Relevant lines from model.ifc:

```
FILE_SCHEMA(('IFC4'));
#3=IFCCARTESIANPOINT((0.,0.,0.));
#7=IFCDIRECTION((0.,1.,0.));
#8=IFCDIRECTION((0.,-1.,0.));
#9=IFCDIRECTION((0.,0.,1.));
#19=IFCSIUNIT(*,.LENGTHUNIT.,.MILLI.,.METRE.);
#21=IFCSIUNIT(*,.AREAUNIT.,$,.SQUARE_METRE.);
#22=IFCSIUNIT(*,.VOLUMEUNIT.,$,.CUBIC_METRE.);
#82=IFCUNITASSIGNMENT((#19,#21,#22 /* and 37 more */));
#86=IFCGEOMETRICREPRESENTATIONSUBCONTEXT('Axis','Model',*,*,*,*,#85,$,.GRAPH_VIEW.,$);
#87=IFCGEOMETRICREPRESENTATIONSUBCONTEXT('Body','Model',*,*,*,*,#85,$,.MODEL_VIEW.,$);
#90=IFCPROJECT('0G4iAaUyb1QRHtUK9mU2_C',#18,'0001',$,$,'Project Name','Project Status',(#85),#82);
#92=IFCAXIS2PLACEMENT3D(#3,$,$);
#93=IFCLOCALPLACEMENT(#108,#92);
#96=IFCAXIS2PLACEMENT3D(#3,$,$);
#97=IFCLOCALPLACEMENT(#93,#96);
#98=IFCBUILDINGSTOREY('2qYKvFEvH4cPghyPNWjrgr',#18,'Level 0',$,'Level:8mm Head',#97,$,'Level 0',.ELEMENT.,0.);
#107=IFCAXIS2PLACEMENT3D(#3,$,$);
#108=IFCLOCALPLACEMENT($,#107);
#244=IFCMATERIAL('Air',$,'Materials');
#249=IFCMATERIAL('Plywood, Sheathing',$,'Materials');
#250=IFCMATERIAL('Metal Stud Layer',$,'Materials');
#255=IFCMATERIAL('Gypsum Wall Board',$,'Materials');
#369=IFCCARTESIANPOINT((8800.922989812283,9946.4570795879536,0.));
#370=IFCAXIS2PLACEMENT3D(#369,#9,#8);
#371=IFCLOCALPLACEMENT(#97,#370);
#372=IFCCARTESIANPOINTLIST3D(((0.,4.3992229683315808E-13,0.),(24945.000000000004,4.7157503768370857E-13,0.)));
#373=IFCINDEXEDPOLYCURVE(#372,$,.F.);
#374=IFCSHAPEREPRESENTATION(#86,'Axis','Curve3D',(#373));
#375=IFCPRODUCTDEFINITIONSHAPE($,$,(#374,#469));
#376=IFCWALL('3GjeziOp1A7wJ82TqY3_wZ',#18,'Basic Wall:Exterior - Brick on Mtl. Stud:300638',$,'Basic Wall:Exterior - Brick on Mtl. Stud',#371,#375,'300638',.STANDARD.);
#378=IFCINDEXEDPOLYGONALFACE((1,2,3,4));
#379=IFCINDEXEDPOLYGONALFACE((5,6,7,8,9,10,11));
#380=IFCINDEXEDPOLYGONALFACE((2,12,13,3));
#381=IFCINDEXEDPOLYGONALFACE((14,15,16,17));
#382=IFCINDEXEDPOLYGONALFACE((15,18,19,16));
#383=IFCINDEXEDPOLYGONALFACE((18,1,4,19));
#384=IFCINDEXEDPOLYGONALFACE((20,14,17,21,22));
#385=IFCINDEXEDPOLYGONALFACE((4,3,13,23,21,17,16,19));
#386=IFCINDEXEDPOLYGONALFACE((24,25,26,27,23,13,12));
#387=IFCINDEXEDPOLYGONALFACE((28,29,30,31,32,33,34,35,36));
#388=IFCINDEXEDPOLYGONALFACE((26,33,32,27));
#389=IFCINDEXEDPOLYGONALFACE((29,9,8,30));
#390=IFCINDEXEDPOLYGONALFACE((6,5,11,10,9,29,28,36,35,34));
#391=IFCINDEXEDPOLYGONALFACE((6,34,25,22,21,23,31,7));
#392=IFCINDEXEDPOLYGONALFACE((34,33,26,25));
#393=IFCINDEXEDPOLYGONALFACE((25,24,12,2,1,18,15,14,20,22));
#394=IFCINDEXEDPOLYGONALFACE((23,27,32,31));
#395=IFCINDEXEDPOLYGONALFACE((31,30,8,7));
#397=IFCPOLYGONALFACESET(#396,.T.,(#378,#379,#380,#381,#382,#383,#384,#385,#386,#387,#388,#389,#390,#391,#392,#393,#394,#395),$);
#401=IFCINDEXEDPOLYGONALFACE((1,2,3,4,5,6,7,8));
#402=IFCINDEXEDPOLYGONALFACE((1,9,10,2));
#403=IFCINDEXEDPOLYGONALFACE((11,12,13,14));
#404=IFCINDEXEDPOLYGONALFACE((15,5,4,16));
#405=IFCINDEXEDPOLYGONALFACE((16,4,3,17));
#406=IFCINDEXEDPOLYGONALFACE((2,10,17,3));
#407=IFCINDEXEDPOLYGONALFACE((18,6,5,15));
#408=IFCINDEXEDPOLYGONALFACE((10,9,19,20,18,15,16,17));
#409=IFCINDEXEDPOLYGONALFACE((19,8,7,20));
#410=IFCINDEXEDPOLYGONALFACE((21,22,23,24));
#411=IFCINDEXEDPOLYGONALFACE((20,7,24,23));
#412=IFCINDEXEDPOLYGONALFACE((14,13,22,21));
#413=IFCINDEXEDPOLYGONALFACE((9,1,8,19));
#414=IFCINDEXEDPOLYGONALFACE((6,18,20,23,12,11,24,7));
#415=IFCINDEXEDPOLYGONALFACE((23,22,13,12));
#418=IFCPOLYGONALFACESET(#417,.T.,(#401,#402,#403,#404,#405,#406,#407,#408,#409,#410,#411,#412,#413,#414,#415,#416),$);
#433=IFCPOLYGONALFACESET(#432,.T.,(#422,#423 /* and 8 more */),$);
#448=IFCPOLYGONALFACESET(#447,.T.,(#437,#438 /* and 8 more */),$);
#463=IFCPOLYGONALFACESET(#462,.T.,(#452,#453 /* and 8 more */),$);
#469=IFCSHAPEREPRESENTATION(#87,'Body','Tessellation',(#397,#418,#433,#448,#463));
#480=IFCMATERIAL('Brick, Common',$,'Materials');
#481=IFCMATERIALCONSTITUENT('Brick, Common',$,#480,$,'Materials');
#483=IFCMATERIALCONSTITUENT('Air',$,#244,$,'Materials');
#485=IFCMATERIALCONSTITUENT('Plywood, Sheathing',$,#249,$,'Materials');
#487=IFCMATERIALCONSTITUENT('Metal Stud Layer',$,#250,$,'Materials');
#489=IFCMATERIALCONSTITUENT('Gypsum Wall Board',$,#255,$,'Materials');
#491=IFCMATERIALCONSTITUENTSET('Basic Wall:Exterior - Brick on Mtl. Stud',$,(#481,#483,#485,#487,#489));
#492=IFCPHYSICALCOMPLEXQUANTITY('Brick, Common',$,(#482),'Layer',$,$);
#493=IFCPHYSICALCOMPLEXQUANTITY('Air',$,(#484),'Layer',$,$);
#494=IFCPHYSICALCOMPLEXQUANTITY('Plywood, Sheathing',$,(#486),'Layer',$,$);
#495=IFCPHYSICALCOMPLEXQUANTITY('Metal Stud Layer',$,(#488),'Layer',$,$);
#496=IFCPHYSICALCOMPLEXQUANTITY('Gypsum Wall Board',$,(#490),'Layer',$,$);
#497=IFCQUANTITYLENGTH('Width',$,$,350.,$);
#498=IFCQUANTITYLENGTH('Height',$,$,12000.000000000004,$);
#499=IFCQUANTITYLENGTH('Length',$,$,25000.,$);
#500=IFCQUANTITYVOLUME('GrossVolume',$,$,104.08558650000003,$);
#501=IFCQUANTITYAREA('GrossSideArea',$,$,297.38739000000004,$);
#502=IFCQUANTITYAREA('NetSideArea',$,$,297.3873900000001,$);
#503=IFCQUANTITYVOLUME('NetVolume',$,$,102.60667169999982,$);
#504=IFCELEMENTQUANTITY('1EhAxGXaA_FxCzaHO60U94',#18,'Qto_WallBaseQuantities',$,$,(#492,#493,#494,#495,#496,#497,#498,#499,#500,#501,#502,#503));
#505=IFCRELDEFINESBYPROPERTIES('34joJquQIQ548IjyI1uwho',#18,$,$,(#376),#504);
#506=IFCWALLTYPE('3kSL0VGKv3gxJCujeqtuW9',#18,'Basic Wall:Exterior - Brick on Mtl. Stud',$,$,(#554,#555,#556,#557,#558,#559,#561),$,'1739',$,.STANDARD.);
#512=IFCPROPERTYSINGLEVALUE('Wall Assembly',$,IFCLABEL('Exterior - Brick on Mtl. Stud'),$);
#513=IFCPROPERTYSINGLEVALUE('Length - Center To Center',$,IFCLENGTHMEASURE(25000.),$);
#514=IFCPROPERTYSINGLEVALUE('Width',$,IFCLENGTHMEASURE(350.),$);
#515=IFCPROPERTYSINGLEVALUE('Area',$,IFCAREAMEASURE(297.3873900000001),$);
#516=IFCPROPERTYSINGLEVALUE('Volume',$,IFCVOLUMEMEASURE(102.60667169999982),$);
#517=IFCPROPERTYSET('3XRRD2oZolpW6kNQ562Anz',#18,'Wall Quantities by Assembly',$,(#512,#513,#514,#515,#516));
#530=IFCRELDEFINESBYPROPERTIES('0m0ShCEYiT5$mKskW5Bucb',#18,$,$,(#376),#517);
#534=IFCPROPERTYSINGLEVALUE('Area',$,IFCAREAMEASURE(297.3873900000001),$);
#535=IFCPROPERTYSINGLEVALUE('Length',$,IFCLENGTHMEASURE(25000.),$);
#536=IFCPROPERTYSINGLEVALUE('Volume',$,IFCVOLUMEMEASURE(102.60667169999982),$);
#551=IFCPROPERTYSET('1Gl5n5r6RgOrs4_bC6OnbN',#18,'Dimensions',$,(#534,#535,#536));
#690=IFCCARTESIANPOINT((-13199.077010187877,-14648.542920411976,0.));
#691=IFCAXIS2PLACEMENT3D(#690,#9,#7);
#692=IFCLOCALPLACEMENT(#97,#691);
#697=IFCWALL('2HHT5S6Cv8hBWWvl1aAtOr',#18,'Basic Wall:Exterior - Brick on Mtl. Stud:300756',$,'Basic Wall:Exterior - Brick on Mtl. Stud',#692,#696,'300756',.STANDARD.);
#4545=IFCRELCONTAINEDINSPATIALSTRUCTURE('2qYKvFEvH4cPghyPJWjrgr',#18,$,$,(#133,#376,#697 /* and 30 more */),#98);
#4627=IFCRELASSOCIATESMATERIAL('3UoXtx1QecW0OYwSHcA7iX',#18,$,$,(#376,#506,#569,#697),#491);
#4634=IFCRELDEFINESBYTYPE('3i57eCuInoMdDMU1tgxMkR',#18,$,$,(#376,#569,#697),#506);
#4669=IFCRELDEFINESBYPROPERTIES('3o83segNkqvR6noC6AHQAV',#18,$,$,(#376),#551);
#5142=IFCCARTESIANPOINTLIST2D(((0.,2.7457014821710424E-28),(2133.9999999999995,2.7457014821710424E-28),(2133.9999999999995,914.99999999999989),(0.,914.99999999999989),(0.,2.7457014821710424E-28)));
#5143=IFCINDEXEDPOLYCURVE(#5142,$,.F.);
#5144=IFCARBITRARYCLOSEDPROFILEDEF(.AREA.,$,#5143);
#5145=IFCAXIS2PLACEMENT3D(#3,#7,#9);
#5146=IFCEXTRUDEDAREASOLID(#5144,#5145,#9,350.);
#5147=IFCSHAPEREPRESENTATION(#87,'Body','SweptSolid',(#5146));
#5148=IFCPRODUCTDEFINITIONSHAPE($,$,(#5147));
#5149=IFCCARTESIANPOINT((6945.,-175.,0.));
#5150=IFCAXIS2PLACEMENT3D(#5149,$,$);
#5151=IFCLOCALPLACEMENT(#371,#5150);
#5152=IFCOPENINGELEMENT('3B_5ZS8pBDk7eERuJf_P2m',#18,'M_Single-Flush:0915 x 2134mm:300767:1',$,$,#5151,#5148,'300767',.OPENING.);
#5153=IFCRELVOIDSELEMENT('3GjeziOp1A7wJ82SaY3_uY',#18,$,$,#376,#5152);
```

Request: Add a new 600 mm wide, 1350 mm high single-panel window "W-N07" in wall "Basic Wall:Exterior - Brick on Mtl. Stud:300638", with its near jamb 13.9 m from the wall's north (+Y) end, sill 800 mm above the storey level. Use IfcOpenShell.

```python
import numpy as np
import ifcopenshell
import ifcopenshell.api.feature
import ifcopenshell.api.geometry
import ifcopenshell.api.pset
import ifcopenshell.api.root
import ifcopenshell.api.spatial
import ifcopenshell.geom
import ifcopenshell.util.element
import ifcopenshell.util.placement
import ifcopenshell.util.representation
import ifcopenshell.util.shape
import ifcopenshell.util.unit

model = ifcopenshell.open("model.ifc")
unit_scale = ifcopenshell.util.unit.calculate_unit_scale(model)
area_scale = ifcopenshell.util.unit.calculate_unit_scale(model, "AREAUNIT")
volume_scale = ifcopenshell.util.unit.calculate_unit_scale(model, "VOLUMEUNIT")
settings = ifcopenshell.geom.settings()


def volume(element):
    """Net volume in cubic metres, openings subtracted."""
    shape = ifcopenshell.geom.create_shape(settings, element)
    return ifcopenshell.util.shape.get_volume(shape.geometry)


wall = model.by_id(376)
storey = ifcopenshell.util.element.get_container(wall, ifc_class="IfcBuildingStorey")
context = ifcopenshell.util.representation.get_context(model, "Model", "Body", "MODEL_VIEW")
before = volume(wall)

width, height, from_end, sill = 0.6, 1.35, 13.9, 0.8  # metres

# The wall runs along its own X axis, and the end named is its -X end.
wall_shape = ifcopenshell.geom.create_shape(settings, wall)
x, y, z = ifcopenshell.util.shape.get_vertices(wall_shape.geometry).T
start = x.min() + from_end
face, thickness = float(y.min()), float(y.max() - y.min())
wall_matrix = ifcopenshell.util.placement.get_local_placement(wall.ObjectPlacement)
level = ifcopenshell.util.placement.get_local_placement(storey.ObjectPlacement)[2, 3]


def in_wall(x, y):
    """Placement at x, y metres in the wall's axes, at sill height."""
    matrix = wall_matrix.copy()
    matrix[:, 3] = wall_matrix @ np.array([x / unit_scale, y / unit_scale, 0.0, 1.0])
    matrix[2, 3] = level + sill / unit_scale
    return matrix


# Opening: a box that overshoots both wall faces by 50 mm.
opening = ifcopenshell.api.root.create_entity(model, ifc_class="IfcOpeningElement", predefined_type="OPENING")
box = ifcopenshell.api.geometry.add_wall_representation(
    model, context=context, length=width, height=height, thickness=thickness + 0.1
)
ifcopenshell.api.geometry.assign_representation(model, product=opening, representation=box)
ifcopenshell.api.geometry.edit_object_placement(model, product=opening, matrix=in_wall(start, face - 0.05), is_si=False)
ifcopenshell.api.feature.add_feature(model, feature=opening, element=wall)

window = ifcopenshell.api.root.create_entity(model, ifc_class="IfcWindow", name="W-N07", predefined_type="WINDOW")
window.OverallWidth, window.OverallHeight = width / unit_scale, height / unit_scale
window.PartitioningType = "SINGLE_PANEL"
body = ifcopenshell.api.geometry.add_window_representation(
    model,
    context=context,
    overall_width=window.OverallWidth,
    overall_height=window.OverallHeight,
    partition_type="SINGLE_PANEL",
)
ifcopenshell.api.geometry.assign_representation(model, product=window, representation=body)
ifcopenshell.api.spatial.assign_container(model, products=[window], relating_structure=storey)
ifcopenshell.api.feature.add_filling(model, opening=opening, element=window)

# Centre the window in the wall's thickness.
ifcopenshell.api.geometry.edit_object_placement(model, product=window, matrix=in_wall(start, face), is_si=False)
window_shape = ifcopenshell.geom.create_shape(settings, window)
depth = ifcopenshell.util.shape.get_vertices(window_shape.geometry)[:, 1]
offset = face + thickness / 2 - (depth.min() + depth.max()) / 2
ifcopenshell.api.geometry.edit_object_placement(model, product=window, matrix=in_wall(start, offset), is_si=False)

after = volume(wall)

# Update the wall's stored quantities.
qto = model.by_id(ifcopenshell.util.element.get_pset(wall, "Qto_WallBaseQuantities", should_inherit=False)["id"])
ifcopenshell.api.pset.edit_qto(model, qto=qto, properties={
    "NetSideArea": after / thickness / area_scale,
    "NetVolume": after / volume_scale,
})
pset = model.by_id(ifcopenshell.util.element.get_pset(wall, "Wall Quantities by Assembly", should_inherit=False)["id"])
ifcopenshell.api.pset.edit_pset(model, pset=pset, properties={
    "Area": model.create_entity("IfcAreaMeasure", after / thickness / area_scale),
    "Volume": model.create_entity("IfcVolumeMeasure", after / volume_scale),
})
pset = model.by_id(ifcopenshell.util.element.get_pset(wall, "Dimensions", should_inherit=False)["id"])
ifcopenshell.api.pset.edit_pset(model, pset=pset, properties={
    "Area": model.create_entity("IfcAreaMeasure", after / thickness / area_scale),
    "Volume": model.create_entity("IfcVolumeMeasure", after / volume_scale),
})

print(f"wall volume {before:.3f} -> {after:.3f} m3")

model.write("model_updated.ifc")
```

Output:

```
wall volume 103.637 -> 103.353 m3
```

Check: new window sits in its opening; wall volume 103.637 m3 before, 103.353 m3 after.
